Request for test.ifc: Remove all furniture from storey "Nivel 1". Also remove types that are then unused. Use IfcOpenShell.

First a look at what the model holds.

```python
import ifcopenshell
import ifcopenshell.util.element

model = ifcopenshell.open("test.ifc")
print(model.schema)
storey = next(s for s in model.by_type("IfcBuildingStorey") if s.Name == "Nivel 1")
furniture = [e for e in ifcopenshell.util.element.get_decomposition(storey) if e.is_a("IfcFurnishingElement")]
seen = {}
for e in furniture:
    element_type = ifcopenshell.util.element.get_type(e)
    name = element_type.Name if element_type not in (None, e) else None
    seen[name] = seen.get(name, 0) + 1
for name, count in sorted(seen.items(), key=str):
    print(count, "x", name)
```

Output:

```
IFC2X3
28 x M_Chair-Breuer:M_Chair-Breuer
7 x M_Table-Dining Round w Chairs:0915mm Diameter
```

```python
import ifcopenshell
import ifcopenshell.api.root
import ifcopenshell.util.element

model = ifcopenshell.open("test.ifc")

storey = next(s for s in model.by_type("IfcBuildingStorey") if s.Name == "Nivel 1")
furniture = [e for e in ifcopenshell.util.element.get_decomposition(storey) if e.is_a("IfcFurnishingElement")]
types = {ifcopenshell.util.element.get_type(e) for e in furniture} - {None, *furniture}

for e in furniture:
    ifcopenshell.api.root.remove_product(model, product=e)
print(len(furniture), "removed")

unused = [t for t in types if not ifcopenshell.util.element.get_types(t)]
for t in unused:
    ifcopenshell.api.root.remove_product(model, product=t)
print(len(unused), "unused types removed")

model.write("test_rev.ifc")
```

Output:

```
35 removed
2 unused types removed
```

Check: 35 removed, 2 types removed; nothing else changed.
